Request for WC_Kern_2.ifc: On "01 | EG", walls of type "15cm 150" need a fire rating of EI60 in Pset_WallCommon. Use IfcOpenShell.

First a look at what the model holds.

```python
import ifcopenshell
import ifcopenshell.util.element

model = ifcopenshell.open("WC_Kern_2.ifc")
print(model.schema)
storey = next(s for s in model.by_type("IfcBuildingStorey") if s.Name == "01 | EG")
walls = [e for e in ifcopenshell.util.element.get_decomposition(storey) if e.is_a("IfcWall")]
seen = {}
for e in walls:
    element_type = ifcopenshell.util.element.get_type(e)
    key = (element_type.Name if element_type != e and element_type else None, ifcopenshell.util.element.get_pset(e, "Pset_WallCommon", "FireRating"))
    seen[key] = seen.get(key, 0) + 1
for (name, value), count in sorted(seen.items(), key=str):
    print(count, "x", name, "|", value)
```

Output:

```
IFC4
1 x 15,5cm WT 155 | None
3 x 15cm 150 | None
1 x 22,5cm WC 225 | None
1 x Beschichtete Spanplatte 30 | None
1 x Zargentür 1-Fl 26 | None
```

```python
import ifcopenshell
import ifcopenshell.api.pset
import ifcopenshell.util.element

model = ifcopenshell.open("WC_Kern_2.ifc")

storey = next(s for s in model.by_type("IfcBuildingStorey") if s.Name == "01 | EG")
walls = [e for e in ifcopenshell.util.element.get_decomposition(storey) if e.is_a("IfcWall")]

count = 0
for e in walls:
    element_type = ifcopenshell.util.element.get_type(e)
    if element_type in (None, e) or element_type.Name != "15cm 150":
        continue
    # add_pset returns the element's existing set when there is one.
    pset = ifcopenshell.api.pset.add_pset(model, product=e, name="Pset_WallCommon")
    ifcopenshell.api.pset.edit_pset(model, pset=pset, properties={"FireRating": "EI60"})
    count += 1

print(count, "walls updated")

model.write("WC_Kern_2_edited.ifc")
```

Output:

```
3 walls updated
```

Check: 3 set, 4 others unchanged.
